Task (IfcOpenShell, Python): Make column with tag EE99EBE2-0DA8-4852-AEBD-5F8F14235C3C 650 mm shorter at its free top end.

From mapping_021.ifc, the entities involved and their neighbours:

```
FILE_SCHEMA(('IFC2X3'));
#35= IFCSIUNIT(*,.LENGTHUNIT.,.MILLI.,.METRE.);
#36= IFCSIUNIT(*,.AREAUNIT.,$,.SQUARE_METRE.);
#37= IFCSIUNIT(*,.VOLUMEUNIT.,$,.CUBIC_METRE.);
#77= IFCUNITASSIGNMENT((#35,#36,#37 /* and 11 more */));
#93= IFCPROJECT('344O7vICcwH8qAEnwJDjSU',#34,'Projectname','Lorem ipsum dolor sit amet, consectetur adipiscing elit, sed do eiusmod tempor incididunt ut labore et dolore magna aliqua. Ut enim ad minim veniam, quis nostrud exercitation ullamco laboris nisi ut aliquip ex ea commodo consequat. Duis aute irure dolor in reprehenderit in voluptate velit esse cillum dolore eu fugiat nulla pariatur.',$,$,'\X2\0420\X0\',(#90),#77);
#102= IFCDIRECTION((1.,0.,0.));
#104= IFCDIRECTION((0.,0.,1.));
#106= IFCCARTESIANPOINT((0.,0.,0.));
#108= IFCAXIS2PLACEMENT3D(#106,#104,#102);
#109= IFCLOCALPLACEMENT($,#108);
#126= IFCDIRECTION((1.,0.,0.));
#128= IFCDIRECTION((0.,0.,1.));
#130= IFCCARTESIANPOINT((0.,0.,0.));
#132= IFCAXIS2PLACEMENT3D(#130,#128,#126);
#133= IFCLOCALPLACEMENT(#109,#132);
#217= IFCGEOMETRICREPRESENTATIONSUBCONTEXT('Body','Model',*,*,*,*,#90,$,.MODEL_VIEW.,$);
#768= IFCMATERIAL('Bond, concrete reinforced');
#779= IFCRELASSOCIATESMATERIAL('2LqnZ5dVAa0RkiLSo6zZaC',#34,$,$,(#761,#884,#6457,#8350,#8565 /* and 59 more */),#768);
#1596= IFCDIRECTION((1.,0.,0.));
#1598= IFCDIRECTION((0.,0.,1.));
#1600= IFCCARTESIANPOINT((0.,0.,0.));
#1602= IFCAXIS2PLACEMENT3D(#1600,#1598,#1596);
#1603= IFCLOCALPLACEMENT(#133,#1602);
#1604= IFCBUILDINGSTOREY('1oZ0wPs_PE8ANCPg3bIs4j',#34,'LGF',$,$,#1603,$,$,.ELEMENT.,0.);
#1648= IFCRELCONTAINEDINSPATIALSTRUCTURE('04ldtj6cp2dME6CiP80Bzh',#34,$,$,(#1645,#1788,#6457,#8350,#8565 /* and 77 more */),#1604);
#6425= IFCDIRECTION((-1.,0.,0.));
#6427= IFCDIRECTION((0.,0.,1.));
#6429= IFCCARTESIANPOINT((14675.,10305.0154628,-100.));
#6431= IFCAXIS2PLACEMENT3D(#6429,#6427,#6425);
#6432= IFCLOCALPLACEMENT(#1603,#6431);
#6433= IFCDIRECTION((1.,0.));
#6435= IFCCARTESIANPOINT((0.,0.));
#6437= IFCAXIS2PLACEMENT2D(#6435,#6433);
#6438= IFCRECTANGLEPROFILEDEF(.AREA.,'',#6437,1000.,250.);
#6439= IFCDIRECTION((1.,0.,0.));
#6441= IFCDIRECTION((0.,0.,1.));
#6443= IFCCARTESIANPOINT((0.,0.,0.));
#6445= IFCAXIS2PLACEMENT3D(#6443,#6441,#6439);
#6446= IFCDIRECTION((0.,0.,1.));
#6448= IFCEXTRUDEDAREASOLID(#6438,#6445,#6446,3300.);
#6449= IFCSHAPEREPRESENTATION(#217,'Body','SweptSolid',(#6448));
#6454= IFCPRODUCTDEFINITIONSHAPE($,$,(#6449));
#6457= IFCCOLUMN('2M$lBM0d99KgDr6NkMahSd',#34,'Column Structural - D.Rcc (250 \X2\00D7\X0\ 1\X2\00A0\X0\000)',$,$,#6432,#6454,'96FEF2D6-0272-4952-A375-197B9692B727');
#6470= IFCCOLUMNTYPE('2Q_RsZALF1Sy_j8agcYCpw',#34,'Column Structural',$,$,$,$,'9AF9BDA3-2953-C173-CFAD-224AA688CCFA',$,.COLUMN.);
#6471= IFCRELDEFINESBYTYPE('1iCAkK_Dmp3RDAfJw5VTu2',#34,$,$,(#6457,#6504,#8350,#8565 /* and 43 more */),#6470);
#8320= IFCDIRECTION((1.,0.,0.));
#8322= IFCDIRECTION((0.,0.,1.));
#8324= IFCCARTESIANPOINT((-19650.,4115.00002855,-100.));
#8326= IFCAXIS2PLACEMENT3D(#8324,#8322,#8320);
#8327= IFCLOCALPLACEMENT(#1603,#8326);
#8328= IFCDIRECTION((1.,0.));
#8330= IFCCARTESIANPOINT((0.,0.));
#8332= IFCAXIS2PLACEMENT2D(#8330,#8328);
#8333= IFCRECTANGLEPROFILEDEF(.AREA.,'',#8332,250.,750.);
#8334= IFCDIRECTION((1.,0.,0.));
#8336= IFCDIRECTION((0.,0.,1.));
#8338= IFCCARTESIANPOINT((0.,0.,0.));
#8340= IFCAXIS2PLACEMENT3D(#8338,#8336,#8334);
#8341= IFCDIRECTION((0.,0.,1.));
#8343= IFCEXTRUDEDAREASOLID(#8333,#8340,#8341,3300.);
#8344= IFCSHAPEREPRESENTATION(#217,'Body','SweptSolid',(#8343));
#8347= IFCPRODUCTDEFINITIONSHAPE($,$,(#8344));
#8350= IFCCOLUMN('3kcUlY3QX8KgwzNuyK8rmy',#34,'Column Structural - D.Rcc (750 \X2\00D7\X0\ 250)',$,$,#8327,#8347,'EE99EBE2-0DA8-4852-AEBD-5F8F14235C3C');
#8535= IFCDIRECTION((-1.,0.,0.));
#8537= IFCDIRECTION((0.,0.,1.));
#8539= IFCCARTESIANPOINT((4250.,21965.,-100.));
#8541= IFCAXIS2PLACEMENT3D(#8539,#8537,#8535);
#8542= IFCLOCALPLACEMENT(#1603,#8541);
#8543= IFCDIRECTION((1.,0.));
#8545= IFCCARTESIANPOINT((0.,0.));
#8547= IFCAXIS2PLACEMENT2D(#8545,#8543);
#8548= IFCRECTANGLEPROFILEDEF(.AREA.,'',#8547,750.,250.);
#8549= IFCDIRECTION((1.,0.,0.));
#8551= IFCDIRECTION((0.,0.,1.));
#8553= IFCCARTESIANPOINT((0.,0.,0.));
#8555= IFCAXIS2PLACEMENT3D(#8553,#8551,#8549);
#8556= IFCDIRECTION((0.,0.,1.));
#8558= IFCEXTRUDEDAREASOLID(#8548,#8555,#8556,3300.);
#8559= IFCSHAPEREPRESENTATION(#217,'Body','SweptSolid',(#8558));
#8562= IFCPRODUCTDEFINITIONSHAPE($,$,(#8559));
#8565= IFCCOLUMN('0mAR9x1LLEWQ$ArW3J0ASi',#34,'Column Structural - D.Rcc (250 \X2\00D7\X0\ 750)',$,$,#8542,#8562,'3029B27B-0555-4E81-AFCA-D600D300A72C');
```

```python
import ifcopenshell
import ifcopenshell.util.representation
import ifcopenshell.util.unit

model = ifcopenshell.open("mapping_021.ifc")
unit_scale = ifcopenshell.util.unit.calculate_unit_scale(model)

member = model.by_id(8350)
change = -0.65 / unit_scale

# The extrusion runs towards the end named, so only its depth changes.
body = ifcopenshell.util.representation.get_representation(member, "Model", "Body")
solid = body.Items[0]
old_length = solid.Depth
solid.Depth += change

print(f"length {old_length:g} -> {solid.Depth:g}")

model.write("mapping_021_v2.ifc")
```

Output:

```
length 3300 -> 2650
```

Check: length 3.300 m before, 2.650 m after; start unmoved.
